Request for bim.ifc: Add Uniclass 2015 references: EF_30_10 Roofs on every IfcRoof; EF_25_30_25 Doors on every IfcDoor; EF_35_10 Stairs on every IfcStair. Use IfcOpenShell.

First a look at what the model holds.

```python
import ifcopenshell

model = ifcopenshell.open("bim.ifc")
print(model.schema)
print("classifications:", [c.Name for c in model.by_type("IfcClassification")])
for ifc_class in ("IfcDoor", "IfcRoof", "IfcStair", "IfcWall", "IfcWindow"):
    print(ifc_class, len(model.by_type(ifc_class)))
```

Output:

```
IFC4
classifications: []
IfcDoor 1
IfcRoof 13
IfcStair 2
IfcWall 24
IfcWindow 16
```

```python
import ifcopenshell
import ifcopenshell.api.classification

model = ifcopenshell.open("bim.ifc")

system = ifcopenshell.api.classification.add_classification(model, classification="Uniclass 2015")

codes = {
    "IfcRoof": ("EF_30_10", "Roofs"),
    "IfcDoor": ("EF_25_30_25", "Doors"),
    "IfcStair": ("EF_35_10", "Stairs"),
}
for ifc_class, (code, name) in codes.items():
    products = model.by_type(ifc_class)
    ifcopenshell.api.classification.add_reference(
        model, products=products, classification=system, identification=code, name=name
    )
    print(code, len(products))

model.write("bim_rev.ifc")
```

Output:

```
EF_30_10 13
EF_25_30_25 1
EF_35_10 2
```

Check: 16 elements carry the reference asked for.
